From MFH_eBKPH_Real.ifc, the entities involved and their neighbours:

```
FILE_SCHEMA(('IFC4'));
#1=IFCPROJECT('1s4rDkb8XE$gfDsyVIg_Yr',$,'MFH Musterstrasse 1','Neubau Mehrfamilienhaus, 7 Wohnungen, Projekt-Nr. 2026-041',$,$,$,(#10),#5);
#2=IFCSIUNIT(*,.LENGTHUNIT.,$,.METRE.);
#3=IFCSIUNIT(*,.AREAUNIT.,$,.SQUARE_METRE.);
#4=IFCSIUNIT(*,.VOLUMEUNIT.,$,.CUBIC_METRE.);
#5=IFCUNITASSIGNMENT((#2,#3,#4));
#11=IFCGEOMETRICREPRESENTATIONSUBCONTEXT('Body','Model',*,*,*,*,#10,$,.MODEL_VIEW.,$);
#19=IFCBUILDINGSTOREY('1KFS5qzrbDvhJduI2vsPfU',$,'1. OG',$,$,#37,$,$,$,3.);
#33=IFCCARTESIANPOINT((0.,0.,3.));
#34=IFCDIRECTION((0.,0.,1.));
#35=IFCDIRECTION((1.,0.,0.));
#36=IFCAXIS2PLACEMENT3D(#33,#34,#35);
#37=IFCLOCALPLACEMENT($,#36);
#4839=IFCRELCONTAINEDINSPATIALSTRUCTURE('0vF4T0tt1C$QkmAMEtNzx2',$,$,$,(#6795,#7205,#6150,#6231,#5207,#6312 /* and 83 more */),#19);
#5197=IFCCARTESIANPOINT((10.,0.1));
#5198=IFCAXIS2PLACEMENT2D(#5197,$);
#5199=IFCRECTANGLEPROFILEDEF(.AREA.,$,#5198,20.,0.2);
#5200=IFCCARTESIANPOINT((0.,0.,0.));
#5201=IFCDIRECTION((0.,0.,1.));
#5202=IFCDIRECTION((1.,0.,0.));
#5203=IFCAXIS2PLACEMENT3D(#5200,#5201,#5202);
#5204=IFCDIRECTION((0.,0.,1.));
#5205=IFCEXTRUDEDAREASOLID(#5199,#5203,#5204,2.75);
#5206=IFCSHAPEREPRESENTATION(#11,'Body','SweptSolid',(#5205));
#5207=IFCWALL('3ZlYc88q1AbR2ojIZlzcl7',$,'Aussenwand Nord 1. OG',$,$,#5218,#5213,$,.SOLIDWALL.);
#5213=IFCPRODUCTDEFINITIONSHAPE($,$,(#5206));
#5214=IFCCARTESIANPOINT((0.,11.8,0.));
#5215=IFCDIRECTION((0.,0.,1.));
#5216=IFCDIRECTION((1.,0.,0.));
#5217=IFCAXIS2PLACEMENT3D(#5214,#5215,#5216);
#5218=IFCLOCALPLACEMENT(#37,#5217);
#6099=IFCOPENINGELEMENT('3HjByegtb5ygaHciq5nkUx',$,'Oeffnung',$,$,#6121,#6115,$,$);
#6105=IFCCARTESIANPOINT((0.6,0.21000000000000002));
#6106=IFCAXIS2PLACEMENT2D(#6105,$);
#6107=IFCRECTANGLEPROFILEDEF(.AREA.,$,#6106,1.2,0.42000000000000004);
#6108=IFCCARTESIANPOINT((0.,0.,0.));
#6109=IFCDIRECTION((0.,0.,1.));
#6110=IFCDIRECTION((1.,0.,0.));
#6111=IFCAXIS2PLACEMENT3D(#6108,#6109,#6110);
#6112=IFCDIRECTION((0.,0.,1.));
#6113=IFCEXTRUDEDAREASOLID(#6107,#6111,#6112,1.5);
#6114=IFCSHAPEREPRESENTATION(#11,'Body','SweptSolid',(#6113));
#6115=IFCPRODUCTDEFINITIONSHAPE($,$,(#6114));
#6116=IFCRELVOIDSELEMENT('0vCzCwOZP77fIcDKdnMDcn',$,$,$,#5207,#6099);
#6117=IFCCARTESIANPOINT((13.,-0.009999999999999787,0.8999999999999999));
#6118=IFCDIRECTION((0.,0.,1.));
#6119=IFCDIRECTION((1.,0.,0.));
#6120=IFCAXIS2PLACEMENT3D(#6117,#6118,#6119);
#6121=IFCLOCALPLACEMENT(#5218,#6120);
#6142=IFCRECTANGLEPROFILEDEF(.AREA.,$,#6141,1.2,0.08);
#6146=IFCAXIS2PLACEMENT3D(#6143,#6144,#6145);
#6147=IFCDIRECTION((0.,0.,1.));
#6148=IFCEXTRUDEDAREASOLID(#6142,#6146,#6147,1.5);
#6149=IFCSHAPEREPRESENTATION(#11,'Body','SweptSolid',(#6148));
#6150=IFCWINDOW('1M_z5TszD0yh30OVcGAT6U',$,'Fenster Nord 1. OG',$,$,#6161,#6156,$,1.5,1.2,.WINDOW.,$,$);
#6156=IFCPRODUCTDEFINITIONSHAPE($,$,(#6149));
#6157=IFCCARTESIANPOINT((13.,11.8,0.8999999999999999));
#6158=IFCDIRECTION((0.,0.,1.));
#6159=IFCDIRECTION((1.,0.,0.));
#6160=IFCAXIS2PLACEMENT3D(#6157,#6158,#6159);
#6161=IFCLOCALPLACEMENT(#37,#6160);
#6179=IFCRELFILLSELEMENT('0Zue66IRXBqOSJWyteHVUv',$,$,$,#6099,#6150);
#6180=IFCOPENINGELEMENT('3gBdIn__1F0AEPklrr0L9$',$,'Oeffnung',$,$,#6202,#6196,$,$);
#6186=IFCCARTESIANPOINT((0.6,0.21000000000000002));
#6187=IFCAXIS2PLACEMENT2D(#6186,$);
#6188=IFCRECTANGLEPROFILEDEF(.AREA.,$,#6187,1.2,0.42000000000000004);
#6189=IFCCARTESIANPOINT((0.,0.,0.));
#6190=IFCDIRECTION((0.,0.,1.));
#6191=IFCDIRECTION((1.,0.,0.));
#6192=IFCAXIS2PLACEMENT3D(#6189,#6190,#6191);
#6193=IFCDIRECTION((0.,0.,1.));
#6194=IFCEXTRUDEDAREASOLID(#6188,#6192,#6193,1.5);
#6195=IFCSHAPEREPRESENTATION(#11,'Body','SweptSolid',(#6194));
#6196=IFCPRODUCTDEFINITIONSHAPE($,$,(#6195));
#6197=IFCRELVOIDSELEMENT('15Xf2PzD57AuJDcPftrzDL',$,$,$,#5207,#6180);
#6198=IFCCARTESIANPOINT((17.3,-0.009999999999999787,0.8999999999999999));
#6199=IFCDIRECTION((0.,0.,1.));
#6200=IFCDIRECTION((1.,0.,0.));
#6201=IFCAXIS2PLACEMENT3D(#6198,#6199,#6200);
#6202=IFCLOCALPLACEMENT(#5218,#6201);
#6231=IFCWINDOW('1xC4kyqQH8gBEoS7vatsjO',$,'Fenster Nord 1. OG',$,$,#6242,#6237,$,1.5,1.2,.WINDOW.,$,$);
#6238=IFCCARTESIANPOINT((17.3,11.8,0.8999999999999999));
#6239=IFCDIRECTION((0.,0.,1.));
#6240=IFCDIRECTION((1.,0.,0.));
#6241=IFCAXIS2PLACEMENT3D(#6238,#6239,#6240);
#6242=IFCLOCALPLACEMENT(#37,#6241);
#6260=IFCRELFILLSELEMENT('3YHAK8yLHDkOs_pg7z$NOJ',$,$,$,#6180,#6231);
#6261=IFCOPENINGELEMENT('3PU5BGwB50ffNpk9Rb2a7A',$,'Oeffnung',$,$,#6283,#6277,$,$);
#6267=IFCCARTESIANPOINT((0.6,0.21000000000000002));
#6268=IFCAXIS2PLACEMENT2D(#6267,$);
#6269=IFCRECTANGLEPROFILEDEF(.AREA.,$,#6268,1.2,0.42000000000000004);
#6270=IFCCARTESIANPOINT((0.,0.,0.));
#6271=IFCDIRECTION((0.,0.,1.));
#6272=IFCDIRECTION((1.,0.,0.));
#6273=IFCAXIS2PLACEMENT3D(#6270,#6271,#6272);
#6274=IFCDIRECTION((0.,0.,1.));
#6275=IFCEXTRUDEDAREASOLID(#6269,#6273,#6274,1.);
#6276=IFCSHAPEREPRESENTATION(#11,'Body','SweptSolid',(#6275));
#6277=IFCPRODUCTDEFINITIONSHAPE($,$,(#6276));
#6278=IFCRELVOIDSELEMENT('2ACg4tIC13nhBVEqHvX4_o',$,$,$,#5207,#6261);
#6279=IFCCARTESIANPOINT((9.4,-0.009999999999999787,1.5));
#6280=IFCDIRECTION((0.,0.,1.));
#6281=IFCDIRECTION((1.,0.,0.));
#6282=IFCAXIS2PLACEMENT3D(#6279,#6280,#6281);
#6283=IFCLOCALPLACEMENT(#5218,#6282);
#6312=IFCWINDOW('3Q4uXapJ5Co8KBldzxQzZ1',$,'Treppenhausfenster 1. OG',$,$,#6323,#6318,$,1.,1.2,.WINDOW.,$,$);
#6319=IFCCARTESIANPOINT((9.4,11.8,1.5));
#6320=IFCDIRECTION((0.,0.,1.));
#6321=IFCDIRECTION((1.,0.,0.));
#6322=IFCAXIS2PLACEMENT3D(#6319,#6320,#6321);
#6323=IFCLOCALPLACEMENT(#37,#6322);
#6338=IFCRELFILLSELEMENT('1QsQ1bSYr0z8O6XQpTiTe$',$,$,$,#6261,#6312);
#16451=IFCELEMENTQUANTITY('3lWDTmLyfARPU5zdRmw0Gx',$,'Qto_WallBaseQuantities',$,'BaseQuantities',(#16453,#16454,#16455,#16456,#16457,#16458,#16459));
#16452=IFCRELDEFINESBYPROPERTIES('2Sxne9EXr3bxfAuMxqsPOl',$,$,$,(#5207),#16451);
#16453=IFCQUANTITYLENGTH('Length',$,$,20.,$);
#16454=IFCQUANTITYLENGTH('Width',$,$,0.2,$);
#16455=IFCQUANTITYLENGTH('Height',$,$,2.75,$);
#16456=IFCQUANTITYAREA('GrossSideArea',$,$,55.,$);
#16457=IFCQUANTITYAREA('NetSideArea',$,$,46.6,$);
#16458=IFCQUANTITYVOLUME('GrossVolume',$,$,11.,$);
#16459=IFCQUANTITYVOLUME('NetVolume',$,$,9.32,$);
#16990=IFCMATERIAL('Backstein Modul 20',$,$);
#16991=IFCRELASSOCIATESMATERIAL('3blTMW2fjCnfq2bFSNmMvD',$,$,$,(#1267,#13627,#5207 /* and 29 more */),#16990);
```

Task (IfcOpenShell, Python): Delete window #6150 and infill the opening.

```python
import ifcopenshell
import ifcopenshell.api.feature
import ifcopenshell.api.pset
import ifcopenshell.api.root
import ifcopenshell.geom
import ifcopenshell.util.element
import ifcopenshell.util.shape
import ifcopenshell.util.unit

model = ifcopenshell.open("MFH_eBKPH_Real.ifc")
area_scale = ifcopenshell.util.unit.calculate_unit_scale(model, "AREAUNIT")
volume_scale = ifcopenshell.util.unit.calculate_unit_scale(model, "VOLUMEUNIT")
settings = ifcopenshell.geom.settings()


def volume(element):
    """Net volume in cubic metres, openings subtracted."""
    shape = ifcopenshell.geom.create_shape(settings, element)
    return ifcopenshell.util.shape.get_volume(shape.geometry)


window = model.by_guid("1M_z5TszD0yh30OVcGAT6U")
opening = window.FillsVoids[0].RelatingOpeningElement
wall = opening.VoidsElements[0].RelatingBuildingElement
before = volume(wall)

ifcopenshell.api.root.remove_product(model, product=window)
ifcopenshell.api.feature.remove_feature(model, feature=opening)

after = volume(wall)
thickness = 0.2  # wall thickness in metres

# Update the wall's stored quantities.
qto = model.by_id(ifcopenshell.util.element.get_pset(wall, "Qto_WallBaseQuantities", should_inherit=False)["id"])
ifcopenshell.api.pset.edit_qto(model, qto=qto, properties={
    "NetSideArea": after / thickness / area_scale,
    "NetVolume": after / volume_scale,
})

print(f"wall volume {before:.3f} -> {after:.3f} m3")

model.write("MFH_eBKPH_Real_rev.ifc")
```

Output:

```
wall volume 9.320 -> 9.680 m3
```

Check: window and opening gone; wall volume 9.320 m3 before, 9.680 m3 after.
